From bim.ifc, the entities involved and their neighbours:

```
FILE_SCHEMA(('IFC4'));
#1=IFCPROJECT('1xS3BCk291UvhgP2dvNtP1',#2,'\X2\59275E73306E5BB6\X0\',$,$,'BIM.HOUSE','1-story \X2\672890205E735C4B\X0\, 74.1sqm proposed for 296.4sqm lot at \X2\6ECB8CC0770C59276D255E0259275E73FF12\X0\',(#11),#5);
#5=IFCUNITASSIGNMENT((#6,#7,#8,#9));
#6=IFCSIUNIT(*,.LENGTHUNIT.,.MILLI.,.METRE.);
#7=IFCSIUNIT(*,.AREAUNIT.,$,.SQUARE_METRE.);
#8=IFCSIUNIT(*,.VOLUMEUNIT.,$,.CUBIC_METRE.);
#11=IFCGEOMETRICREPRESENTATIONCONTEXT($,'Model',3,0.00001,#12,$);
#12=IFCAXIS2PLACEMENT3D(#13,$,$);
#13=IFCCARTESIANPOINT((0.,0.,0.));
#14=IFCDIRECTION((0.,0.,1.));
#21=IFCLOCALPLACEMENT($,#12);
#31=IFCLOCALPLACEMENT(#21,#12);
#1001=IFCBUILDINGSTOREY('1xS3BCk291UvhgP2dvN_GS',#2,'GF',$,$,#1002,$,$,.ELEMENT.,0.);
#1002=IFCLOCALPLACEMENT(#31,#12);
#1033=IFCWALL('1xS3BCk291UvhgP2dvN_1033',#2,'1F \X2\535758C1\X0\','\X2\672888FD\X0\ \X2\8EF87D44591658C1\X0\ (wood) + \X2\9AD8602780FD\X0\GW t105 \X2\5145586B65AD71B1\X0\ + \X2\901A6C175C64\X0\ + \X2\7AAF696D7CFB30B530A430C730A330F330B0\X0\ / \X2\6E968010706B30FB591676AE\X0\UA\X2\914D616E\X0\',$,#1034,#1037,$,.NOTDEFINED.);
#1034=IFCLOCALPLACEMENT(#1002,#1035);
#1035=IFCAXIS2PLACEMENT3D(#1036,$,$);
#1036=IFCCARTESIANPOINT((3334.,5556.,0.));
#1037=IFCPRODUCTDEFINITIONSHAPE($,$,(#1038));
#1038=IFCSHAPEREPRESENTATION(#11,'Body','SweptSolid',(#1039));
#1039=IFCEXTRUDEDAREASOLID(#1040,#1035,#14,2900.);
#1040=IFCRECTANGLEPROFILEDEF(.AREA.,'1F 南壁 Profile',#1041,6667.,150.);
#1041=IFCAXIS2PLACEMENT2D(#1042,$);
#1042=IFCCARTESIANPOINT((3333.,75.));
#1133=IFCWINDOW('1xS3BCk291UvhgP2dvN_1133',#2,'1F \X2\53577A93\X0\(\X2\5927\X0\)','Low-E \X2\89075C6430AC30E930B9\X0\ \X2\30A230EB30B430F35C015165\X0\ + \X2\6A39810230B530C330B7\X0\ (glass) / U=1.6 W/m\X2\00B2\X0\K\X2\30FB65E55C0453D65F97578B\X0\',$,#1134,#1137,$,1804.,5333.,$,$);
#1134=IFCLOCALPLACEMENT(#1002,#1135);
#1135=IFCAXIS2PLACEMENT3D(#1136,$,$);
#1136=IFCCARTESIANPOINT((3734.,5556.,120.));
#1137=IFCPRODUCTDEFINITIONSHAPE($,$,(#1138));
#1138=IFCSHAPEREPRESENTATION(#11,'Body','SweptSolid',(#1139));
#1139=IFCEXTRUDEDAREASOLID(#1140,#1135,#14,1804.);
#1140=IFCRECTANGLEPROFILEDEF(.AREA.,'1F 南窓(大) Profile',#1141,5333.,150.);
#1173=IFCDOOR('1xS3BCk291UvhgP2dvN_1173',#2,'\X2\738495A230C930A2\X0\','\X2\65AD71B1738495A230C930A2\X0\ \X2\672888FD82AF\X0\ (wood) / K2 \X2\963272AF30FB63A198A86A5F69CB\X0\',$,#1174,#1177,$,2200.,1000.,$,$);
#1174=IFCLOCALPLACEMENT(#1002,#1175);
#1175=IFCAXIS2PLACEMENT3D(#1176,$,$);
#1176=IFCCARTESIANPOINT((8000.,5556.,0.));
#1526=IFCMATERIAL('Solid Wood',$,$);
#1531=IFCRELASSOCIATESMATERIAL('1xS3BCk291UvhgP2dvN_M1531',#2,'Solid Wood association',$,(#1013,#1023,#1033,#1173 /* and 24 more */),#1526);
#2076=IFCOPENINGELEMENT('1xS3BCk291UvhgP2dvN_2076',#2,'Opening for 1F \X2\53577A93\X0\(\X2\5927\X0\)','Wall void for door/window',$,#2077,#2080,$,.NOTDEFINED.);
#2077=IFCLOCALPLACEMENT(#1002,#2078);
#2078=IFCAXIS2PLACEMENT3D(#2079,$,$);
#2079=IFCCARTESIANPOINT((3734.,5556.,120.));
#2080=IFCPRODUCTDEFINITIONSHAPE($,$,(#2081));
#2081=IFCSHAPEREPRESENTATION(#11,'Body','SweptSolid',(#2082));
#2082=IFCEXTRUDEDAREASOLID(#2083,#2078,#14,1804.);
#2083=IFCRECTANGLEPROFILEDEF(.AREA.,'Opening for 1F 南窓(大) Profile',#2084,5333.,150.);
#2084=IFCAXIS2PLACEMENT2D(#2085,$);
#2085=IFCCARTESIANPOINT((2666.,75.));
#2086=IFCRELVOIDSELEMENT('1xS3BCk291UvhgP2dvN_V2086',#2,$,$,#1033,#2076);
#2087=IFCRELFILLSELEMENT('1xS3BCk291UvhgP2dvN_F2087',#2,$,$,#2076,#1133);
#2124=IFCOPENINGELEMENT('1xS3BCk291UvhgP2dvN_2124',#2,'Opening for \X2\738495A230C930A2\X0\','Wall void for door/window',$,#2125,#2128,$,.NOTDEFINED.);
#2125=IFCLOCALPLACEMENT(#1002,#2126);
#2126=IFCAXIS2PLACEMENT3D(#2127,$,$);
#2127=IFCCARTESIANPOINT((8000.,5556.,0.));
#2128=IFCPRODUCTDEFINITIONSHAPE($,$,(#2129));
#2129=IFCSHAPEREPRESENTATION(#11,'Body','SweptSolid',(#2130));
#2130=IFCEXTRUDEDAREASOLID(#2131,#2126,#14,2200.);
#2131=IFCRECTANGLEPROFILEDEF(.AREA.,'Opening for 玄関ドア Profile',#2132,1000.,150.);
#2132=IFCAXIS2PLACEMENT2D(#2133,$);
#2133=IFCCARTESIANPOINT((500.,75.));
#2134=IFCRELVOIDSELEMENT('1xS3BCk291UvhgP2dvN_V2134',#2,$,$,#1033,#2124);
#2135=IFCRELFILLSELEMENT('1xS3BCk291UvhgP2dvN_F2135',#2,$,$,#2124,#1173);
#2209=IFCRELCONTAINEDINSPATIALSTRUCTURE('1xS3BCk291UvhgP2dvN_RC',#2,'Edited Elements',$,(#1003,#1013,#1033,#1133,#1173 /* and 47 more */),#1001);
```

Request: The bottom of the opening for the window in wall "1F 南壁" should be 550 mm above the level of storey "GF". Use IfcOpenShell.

```python
import numpy as np
import ifcopenshell
import ifcopenshell.api.geometry
import ifcopenshell.geom
import ifcopenshell.util.element
import ifcopenshell.util.placement
import ifcopenshell.util.shape
import ifcopenshell.util.unit

model = ifcopenshell.open("bim.ifc")
unit_scale = ifcopenshell.util.unit.calculate_unit_scale(model)

window = model.by_id(1133)
opening = window.FillsVoids[0].RelatingOpeningElement
storey = ifcopenshell.util.element.get_container(window, ifc_class="IfcBuildingStorey")
level = ifcopenshell.util.placement.get_local_placement(storey.ObjectPlacement)[2, 3]

# The opening's origin need not be at the sill, so measure its lowest point.
shape = ifcopenshell.geom.create_shape(ifcopenshell.geom.settings(), opening)
bottom = ifcopenshell.util.shape.get_shape_bottom_elevation(shape, shape.geometry) / unit_scale
dz = level + 0.55 / unit_scale - bottom

shift = np.array([0.0, 0.0, dz])
# The window is not placed relative to its opening, so move both.
for product in (opening, window):
    matrix = ifcopenshell.util.placement.get_local_placement(product.ObjectPlacement)
    matrix[:3, 3] += shift
    ifcopenshell.api.geometry.edit_object_placement(model, product=product, matrix=matrix, is_si=False)

print(f"moved by {dz * unit_scale:+.3f} m")

model.write("bim_updated.ifc")
```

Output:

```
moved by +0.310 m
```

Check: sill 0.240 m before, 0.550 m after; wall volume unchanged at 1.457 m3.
